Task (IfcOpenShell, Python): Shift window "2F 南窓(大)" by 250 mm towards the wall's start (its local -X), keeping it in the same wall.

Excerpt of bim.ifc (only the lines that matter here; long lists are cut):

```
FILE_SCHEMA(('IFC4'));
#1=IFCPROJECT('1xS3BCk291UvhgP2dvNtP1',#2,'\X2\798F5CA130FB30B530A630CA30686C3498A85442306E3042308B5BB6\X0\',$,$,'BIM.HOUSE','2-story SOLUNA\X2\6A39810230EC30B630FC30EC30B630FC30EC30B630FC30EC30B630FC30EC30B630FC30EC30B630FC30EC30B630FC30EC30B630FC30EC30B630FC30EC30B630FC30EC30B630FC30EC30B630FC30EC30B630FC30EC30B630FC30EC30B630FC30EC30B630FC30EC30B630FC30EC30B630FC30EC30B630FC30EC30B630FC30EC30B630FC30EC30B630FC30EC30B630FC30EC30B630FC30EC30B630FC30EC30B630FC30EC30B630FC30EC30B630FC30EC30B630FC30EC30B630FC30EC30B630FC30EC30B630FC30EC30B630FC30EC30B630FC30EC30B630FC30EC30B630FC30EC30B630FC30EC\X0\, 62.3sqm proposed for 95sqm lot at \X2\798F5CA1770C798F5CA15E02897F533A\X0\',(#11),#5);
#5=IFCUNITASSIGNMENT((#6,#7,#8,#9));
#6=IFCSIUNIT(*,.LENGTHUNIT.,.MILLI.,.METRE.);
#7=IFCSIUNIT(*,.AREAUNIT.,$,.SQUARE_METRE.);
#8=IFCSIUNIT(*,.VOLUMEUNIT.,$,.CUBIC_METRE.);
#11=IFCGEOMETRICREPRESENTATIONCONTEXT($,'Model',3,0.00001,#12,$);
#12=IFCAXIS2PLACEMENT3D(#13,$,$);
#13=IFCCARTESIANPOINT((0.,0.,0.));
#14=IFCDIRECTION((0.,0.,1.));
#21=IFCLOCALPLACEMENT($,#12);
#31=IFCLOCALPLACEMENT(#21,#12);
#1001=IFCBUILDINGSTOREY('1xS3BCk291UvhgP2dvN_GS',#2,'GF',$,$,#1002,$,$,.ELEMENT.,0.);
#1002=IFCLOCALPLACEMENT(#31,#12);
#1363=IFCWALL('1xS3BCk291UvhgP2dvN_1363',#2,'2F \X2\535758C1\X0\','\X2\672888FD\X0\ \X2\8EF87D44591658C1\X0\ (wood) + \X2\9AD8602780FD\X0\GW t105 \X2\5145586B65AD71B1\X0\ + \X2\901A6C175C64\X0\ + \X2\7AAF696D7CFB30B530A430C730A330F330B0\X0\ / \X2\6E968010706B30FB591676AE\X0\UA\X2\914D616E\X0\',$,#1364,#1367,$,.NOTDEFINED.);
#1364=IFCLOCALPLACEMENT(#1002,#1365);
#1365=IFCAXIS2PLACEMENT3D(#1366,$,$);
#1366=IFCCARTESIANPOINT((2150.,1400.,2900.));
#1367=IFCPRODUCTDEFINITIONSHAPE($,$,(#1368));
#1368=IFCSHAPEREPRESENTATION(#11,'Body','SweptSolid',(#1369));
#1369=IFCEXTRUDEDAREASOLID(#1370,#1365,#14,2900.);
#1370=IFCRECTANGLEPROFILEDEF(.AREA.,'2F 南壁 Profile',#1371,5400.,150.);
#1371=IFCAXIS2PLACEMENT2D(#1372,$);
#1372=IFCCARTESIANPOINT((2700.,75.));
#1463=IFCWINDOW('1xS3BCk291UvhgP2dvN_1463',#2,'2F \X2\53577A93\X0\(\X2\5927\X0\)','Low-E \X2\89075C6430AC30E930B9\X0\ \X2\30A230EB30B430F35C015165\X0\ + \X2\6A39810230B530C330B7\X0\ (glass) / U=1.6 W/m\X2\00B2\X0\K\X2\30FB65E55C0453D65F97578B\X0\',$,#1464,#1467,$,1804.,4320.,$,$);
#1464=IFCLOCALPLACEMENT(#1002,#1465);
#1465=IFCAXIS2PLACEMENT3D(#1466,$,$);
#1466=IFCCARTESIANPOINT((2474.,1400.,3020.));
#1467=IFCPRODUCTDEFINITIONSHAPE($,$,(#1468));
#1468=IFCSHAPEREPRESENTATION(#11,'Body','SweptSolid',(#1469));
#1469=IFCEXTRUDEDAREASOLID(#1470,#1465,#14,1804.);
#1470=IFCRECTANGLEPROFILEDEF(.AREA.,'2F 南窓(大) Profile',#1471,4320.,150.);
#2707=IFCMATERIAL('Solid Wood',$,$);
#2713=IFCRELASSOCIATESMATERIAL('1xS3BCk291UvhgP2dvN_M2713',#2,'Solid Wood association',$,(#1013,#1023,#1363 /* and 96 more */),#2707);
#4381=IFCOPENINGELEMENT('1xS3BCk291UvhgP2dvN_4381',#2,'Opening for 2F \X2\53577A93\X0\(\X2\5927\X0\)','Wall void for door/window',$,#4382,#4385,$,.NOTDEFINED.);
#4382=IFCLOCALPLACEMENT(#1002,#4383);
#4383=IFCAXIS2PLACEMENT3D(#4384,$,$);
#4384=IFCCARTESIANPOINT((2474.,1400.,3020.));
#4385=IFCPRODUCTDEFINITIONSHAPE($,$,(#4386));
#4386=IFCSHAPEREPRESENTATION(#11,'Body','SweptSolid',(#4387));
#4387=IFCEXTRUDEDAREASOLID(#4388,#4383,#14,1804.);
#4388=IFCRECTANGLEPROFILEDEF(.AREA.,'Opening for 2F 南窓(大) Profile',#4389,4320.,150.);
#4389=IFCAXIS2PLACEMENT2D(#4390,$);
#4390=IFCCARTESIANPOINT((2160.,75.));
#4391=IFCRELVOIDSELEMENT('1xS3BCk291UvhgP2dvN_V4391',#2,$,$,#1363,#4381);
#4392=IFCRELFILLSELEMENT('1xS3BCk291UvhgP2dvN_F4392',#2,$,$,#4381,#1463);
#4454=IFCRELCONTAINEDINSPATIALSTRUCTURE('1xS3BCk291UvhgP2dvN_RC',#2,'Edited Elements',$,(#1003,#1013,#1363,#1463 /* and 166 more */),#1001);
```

```python
import ifcopenshell
import ifcopenshell.api.geometry
import ifcopenshell.util.placement

model = ifcopenshell.open("bim.ifc")

window = model.by_id(1463)
opening = window.FillsVoids[0].RelatingOpeningElement
wall = opening.VoidsElements[0].RelatingBuildingElement

wall_matrix = ifcopenshell.util.placement.get_local_placement(wall.ObjectPlacement)
shift = wall_matrix[:3, 0] * -250.0
before = ifcopenshell.util.placement.get_local_placement(window.ObjectPlacement)[:3, 3].copy()

# The window is not placed relative to its opening, so move both.
for product in (opening, window):
    matrix = ifcopenshell.util.placement.get_local_placement(product.ObjectPlacement)
    matrix[:3, 3] += shift
    ifcopenshell.api.geometry.edit_object_placement(model, product=product, matrix=matrix, is_si=False)

after = ifcopenshell.util.placement.get_local_placement(window.ObjectPlacement)[:3, 3]
print("window moved by", (after - before).round(3) + 0.0)

model.write("bim_v2.ifc")
```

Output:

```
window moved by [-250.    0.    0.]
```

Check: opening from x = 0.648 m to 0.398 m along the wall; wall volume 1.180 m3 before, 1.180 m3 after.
